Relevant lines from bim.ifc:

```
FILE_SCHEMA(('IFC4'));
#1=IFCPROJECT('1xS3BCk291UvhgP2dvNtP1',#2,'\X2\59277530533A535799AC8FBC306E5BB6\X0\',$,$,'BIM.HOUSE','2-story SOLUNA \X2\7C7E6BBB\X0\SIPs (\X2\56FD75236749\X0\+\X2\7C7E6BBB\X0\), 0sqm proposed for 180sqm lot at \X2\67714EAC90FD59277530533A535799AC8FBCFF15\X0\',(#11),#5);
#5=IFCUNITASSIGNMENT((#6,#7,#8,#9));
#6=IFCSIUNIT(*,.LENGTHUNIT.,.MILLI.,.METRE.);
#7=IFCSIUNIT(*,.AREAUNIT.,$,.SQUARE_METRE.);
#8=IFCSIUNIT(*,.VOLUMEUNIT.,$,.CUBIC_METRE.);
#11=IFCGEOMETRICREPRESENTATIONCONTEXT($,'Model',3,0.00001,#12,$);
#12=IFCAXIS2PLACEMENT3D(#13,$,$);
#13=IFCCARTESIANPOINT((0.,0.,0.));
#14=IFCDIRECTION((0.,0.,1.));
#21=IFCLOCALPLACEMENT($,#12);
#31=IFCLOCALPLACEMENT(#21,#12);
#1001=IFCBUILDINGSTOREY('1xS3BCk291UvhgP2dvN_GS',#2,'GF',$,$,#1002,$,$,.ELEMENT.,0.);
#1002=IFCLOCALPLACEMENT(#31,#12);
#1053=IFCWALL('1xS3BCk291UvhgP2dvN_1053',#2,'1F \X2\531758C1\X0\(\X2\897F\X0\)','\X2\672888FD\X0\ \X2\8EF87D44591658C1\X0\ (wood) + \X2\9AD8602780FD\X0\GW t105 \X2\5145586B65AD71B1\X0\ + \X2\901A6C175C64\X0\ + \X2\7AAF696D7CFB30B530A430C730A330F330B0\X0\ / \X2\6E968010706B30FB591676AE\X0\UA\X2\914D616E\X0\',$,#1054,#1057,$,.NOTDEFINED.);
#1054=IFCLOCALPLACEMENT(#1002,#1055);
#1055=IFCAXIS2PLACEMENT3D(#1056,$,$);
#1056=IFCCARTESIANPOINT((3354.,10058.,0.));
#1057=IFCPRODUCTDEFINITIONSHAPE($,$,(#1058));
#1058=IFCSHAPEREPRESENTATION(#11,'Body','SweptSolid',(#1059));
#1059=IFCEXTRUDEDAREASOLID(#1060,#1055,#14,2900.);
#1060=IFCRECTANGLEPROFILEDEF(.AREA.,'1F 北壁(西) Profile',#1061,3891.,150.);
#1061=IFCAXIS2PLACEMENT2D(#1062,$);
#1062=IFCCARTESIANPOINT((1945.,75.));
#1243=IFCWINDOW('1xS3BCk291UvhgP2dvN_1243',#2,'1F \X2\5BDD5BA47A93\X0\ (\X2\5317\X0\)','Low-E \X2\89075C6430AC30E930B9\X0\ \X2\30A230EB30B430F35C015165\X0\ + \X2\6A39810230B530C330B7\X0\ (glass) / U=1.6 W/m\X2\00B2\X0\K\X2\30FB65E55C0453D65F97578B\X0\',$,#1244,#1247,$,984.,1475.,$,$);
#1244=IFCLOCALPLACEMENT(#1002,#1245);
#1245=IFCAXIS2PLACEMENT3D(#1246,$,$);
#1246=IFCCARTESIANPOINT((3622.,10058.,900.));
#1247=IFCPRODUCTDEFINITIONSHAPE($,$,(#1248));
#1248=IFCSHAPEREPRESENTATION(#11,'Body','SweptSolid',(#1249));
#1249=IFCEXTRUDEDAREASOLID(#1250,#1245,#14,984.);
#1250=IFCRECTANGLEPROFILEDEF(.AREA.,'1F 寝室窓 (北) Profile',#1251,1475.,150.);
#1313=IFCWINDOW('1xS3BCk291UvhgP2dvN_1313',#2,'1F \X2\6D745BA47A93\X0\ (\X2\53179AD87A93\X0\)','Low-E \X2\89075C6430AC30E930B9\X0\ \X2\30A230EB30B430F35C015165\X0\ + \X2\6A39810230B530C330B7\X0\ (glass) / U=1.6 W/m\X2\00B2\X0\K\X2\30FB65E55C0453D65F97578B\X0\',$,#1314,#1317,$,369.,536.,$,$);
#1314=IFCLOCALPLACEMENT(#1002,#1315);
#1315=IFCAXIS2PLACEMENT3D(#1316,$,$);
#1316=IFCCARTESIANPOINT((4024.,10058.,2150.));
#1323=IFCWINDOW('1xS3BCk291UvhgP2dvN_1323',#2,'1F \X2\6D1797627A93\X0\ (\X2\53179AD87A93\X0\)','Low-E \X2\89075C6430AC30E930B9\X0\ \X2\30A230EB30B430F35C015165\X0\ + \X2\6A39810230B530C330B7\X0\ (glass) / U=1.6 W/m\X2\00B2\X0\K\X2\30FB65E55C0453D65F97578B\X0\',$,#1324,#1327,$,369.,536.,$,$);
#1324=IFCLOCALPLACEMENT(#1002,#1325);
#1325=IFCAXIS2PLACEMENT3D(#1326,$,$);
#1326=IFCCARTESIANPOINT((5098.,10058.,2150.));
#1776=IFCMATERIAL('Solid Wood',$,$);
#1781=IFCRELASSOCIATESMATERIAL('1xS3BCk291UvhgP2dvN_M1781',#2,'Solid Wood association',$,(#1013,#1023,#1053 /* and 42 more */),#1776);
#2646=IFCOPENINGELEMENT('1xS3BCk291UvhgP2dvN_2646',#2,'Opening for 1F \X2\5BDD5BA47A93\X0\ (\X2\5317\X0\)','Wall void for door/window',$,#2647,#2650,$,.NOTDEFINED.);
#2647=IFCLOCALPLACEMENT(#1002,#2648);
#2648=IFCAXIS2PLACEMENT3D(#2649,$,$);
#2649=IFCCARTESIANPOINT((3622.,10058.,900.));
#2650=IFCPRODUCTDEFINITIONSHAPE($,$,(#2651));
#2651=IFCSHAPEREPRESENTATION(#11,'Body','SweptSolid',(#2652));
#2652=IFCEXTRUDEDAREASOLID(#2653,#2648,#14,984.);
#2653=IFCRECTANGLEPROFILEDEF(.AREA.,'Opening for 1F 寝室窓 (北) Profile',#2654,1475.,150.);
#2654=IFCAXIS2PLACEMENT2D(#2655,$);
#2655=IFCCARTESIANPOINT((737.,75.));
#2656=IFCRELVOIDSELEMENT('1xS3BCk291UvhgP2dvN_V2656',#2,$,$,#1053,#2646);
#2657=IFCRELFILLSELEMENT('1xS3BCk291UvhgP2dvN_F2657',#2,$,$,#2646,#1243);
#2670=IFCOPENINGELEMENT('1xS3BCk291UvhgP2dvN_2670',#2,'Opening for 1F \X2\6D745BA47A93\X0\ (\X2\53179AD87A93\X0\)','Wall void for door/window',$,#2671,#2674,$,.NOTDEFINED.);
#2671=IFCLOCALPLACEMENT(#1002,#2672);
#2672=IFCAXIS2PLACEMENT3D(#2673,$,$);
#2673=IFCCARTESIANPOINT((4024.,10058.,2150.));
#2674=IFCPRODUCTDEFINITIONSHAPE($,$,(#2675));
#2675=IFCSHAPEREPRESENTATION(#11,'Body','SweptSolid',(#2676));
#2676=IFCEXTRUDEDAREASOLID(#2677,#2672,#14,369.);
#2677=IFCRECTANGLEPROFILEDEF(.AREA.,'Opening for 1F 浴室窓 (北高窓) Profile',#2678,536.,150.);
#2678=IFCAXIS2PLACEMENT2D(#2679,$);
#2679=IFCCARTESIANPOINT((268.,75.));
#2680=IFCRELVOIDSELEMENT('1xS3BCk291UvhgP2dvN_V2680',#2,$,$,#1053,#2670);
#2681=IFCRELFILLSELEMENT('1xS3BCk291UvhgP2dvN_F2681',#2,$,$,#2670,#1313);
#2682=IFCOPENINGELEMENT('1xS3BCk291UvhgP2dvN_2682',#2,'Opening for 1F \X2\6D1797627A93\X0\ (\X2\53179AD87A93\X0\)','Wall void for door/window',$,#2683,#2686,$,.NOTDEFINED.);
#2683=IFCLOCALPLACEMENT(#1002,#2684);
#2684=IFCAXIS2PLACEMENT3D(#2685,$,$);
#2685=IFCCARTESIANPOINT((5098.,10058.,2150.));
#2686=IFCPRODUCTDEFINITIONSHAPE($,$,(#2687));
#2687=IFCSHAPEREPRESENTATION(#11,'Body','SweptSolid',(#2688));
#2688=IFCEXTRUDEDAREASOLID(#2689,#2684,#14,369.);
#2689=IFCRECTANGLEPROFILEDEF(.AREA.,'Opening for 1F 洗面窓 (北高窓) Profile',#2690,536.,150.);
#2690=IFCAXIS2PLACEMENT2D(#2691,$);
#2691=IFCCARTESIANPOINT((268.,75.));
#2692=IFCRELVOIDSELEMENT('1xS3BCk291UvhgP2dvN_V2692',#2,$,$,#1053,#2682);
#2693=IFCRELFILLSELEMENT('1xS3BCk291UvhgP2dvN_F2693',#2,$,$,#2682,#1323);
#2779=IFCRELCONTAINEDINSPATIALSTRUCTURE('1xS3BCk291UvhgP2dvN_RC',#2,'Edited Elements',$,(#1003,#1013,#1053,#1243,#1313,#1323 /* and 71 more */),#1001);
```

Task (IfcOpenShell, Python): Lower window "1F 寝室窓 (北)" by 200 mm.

```python
import numpy as np
import ifcopenshell
import ifcopenshell.api.geometry
import ifcopenshell.util.placement
import ifcopenshell.util.unit

model = ifcopenshell.open("bim.ifc")
unit_scale = ifcopenshell.util.unit.calculate_unit_scale(model)

window = model.by_guid("1xS3BCk291UvhgP2dvN_1243")
opening = window.FillsVoids[0].RelatingOpeningElement
dz = -200.0

shift = np.array([0.0, 0.0, dz])
# The window is not placed relative to its opening, so move both.
for product in (opening, window):
    matrix = ifcopenshell.util.placement.get_local_placement(product.ObjectPlacement)
    matrix[:3, 3] += shift
    ifcopenshell.api.geometry.edit_object_placement(model, product=product, matrix=matrix, is_si=False)

print(f"moved by {dz * unit_scale:+.3f} m")

model.write("bim_v2.ifc")
```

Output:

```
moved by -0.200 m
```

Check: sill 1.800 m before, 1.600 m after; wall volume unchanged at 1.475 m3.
